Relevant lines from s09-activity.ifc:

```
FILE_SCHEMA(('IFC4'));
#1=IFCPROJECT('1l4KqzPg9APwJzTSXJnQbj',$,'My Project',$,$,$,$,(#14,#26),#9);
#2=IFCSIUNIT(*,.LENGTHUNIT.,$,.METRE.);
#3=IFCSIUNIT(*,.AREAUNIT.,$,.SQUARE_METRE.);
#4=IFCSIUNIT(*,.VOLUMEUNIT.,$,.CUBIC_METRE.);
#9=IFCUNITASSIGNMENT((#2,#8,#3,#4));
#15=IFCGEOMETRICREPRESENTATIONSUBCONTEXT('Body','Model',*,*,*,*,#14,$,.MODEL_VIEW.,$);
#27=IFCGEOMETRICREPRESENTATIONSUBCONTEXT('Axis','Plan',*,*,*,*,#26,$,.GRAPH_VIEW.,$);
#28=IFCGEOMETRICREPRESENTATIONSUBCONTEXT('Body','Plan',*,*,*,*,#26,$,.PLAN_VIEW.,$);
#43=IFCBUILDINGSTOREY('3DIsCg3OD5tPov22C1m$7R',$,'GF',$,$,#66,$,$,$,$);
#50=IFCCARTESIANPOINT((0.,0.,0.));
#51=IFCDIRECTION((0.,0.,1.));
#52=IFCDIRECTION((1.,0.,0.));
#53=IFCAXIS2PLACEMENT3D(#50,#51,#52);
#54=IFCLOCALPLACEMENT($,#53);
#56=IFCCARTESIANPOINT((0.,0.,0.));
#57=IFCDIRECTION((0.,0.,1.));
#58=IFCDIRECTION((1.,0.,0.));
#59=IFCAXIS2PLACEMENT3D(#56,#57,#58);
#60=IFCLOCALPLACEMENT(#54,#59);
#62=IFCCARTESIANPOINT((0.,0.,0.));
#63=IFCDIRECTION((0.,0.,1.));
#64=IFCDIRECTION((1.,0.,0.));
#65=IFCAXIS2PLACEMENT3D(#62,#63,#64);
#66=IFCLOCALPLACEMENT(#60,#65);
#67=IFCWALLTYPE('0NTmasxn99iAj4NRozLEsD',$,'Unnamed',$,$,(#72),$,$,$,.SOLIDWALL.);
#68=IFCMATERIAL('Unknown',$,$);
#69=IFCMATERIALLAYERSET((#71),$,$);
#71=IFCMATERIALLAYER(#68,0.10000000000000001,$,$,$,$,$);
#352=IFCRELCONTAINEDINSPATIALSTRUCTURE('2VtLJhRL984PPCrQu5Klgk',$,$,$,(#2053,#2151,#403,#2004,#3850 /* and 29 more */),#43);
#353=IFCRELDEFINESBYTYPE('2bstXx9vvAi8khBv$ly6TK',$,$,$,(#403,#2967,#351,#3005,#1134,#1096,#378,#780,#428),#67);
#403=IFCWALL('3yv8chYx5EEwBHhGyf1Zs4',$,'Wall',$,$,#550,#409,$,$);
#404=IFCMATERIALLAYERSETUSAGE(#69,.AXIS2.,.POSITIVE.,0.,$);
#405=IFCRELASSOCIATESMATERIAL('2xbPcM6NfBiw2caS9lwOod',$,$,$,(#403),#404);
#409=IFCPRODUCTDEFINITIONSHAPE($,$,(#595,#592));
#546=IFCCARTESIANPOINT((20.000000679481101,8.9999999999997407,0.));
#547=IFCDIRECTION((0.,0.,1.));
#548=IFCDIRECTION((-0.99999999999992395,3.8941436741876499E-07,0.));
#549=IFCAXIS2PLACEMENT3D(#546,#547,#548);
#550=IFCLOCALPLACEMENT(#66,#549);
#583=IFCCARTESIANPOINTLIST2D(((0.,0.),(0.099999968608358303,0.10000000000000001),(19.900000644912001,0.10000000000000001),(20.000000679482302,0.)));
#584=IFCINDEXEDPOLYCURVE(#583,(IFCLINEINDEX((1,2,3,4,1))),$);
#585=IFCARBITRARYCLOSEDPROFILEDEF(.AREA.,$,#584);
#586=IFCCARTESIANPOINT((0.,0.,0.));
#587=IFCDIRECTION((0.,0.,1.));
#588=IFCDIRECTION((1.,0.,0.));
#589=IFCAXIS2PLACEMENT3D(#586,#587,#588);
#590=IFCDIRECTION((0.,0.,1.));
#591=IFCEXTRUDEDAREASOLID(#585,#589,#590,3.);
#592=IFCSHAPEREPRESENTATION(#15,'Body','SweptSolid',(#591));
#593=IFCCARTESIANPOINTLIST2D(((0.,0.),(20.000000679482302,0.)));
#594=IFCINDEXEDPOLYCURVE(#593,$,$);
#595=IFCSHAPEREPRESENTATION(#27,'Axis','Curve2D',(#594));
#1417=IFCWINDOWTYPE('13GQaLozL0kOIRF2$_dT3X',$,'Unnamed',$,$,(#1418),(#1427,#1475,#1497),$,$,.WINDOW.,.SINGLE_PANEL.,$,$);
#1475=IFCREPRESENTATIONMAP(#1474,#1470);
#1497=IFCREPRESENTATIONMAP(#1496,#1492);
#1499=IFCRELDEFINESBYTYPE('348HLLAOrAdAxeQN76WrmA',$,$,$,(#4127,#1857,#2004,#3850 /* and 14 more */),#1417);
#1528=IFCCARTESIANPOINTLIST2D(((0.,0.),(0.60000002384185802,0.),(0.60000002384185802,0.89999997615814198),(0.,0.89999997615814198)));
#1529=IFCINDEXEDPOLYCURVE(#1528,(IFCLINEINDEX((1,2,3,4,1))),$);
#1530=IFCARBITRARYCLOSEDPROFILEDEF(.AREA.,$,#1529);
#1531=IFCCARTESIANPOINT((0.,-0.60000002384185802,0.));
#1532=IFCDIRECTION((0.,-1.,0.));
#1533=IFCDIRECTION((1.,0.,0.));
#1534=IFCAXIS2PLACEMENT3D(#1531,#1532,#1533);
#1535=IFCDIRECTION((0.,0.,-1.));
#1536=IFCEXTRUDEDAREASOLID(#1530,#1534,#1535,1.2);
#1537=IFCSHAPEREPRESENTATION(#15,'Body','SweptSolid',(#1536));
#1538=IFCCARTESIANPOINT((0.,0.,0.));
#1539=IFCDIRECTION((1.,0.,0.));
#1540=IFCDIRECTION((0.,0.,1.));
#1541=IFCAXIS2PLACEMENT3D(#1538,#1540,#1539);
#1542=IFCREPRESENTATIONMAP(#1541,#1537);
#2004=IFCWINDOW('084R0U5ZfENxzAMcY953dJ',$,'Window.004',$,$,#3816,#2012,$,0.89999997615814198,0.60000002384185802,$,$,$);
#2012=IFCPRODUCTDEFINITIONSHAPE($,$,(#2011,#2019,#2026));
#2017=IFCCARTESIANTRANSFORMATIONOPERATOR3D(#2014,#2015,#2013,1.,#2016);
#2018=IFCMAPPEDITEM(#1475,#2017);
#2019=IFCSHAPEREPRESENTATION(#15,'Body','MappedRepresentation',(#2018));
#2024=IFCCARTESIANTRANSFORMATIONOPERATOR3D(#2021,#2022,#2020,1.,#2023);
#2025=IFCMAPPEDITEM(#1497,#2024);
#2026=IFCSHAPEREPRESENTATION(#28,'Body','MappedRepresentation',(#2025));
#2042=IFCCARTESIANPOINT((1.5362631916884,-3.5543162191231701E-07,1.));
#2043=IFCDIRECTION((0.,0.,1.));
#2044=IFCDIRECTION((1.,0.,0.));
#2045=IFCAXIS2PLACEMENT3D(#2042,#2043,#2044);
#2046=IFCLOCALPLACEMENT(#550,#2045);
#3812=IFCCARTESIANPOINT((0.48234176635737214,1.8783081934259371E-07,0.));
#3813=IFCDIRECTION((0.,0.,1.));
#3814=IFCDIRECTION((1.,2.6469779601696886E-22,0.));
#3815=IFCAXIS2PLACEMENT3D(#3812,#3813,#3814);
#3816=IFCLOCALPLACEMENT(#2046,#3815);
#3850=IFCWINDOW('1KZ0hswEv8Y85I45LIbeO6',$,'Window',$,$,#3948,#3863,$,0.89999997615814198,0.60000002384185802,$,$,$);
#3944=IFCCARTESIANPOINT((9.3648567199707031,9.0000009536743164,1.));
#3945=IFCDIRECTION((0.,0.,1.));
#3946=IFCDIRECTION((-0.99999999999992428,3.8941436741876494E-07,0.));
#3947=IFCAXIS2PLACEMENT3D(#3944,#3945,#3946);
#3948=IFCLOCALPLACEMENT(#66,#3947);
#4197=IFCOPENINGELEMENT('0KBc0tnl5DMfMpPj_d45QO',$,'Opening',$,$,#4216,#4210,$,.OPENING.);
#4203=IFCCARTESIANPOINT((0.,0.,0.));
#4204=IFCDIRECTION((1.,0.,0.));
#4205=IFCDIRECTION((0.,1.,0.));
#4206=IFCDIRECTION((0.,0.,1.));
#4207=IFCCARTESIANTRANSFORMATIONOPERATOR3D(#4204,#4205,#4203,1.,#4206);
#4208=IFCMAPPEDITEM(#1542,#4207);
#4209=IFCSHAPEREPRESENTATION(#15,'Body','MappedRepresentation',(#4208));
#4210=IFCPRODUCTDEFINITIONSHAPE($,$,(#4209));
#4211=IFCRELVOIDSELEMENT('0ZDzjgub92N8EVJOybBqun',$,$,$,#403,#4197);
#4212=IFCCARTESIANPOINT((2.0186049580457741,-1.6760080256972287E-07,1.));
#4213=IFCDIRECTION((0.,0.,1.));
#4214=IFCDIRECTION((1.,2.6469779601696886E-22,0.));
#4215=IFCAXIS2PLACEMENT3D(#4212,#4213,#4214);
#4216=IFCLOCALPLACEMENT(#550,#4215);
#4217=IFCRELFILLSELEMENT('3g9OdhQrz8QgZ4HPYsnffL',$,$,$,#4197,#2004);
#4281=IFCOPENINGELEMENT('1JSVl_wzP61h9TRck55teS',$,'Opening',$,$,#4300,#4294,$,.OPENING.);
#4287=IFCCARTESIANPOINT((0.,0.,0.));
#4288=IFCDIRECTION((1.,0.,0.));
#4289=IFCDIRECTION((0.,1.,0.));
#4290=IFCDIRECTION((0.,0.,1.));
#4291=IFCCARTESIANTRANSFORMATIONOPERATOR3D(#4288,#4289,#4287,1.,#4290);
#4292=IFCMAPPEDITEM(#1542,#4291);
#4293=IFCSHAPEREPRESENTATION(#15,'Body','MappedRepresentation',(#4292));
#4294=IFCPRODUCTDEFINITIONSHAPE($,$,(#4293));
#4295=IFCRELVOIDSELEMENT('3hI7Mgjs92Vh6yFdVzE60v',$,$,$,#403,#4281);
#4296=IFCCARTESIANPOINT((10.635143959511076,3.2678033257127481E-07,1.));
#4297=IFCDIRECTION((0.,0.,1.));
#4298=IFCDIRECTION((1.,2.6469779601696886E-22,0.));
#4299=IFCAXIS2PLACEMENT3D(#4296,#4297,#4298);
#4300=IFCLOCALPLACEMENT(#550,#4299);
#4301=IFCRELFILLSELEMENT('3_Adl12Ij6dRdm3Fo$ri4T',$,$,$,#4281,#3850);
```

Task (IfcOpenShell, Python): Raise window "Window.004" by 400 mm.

```python
import numpy as np
import ifcopenshell
import ifcopenshell.api.geometry
import ifcopenshell.util.placement
import ifcopenshell.util.unit

model = ifcopenshell.open("s09-activity.ifc")
unit_scale = ifcopenshell.util.unit.calculate_unit_scale(model)

window = model.by_guid("084R0U5ZfENxzAMcY953dJ")
opening = window.FillsVoids[0].RelatingOpeningElement
dz = 0.4 / unit_scale

shift = np.array([0.0, 0.0, dz])
# The window is not placed relative to its opening, so move both.
for product in (opening, window):
    matrix = ifcopenshell.util.placement.get_local_placement(product.ObjectPlacement)
    matrix[:3, 3] += shift
    ifcopenshell.api.geometry.edit_object_placement(model, product=product, matrix=matrix, is_si=False)

print(f"moved by {dz * unit_scale:+.3f} m")

model.write("s09-activity_updated.ifc")
```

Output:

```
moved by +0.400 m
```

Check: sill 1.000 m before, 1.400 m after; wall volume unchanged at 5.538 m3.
